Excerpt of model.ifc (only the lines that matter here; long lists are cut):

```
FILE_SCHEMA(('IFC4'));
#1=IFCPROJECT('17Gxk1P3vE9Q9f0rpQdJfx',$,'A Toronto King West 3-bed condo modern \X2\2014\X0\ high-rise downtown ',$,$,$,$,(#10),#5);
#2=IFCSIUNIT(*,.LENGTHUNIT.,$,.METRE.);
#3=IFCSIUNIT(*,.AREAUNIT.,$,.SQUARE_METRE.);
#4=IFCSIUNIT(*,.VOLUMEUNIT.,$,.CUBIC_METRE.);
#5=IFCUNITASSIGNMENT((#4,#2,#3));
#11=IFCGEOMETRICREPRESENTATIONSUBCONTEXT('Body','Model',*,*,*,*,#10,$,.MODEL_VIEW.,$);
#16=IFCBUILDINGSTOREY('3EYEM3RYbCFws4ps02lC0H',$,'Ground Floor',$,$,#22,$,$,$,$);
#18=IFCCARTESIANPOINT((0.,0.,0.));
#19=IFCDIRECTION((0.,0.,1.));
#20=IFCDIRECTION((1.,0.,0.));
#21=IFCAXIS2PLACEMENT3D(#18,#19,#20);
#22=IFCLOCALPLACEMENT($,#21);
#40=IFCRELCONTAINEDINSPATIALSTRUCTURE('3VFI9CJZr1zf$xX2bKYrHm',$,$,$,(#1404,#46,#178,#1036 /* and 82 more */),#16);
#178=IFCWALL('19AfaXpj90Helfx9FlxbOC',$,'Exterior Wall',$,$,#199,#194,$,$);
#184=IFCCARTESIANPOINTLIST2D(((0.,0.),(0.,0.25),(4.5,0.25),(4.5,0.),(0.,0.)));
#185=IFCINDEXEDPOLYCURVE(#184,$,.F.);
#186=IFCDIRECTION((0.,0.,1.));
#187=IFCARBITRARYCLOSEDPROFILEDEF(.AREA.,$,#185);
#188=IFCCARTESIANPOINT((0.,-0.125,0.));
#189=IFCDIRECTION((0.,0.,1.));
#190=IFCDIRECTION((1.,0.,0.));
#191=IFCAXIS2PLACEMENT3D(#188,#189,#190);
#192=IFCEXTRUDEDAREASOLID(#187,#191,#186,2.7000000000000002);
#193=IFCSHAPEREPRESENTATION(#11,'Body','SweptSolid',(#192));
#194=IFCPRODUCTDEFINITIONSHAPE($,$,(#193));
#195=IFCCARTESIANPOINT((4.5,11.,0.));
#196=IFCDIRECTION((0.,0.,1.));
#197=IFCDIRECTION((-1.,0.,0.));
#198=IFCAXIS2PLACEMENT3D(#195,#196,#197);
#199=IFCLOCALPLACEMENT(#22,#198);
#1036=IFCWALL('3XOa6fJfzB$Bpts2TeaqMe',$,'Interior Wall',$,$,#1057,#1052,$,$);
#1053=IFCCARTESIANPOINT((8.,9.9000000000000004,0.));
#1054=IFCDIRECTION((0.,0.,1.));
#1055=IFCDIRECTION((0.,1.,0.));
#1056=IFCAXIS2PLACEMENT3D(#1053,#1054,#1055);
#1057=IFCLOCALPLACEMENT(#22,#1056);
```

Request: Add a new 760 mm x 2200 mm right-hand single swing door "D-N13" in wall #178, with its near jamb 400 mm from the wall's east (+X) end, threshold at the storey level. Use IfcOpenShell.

```python
import numpy as np
import ifcopenshell
import ifcopenshell.api.feature
import ifcopenshell.api.geometry
import ifcopenshell.api.root
import ifcopenshell.api.spatial
import ifcopenshell.geom
import ifcopenshell.util.element
import ifcopenshell.util.placement
import ifcopenshell.util.representation
import ifcopenshell.util.shape
import ifcopenshell.util.unit

model = ifcopenshell.open("model.ifc")
unit_scale = ifcopenshell.util.unit.calculate_unit_scale(model)
settings = ifcopenshell.geom.settings()


def volume(element):
    """Net volume in cubic metres, openings subtracted."""
    shape = ifcopenshell.geom.create_shape(settings, element)
    return ifcopenshell.util.shape.get_volume(shape.geometry)


wall = model.by_guid("19AfaXpj90Helfx9FlxbOC")
storey = ifcopenshell.util.element.get_container(wall, ifc_class="IfcBuildingStorey")
context = ifcopenshell.util.representation.get_context(model, "Model", "Body", "MODEL_VIEW")
before = volume(wall)

width, height, from_end, sill = 0.76, 2.2, 0.4, 0.0  # metres

# The wall runs along its own X axis, and the end named is its -X end.
wall_shape = ifcopenshell.geom.create_shape(settings, wall)
x, y, z = ifcopenshell.util.shape.get_vertices(wall_shape.geometry).T
start = x.min() + from_end
face, thickness = float(y.min()), float(y.max() - y.min())
wall_matrix = ifcopenshell.util.placement.get_local_placement(wall.ObjectPlacement)
level = ifcopenshell.util.placement.get_local_placement(storey.ObjectPlacement)[2, 3]


def in_wall(x, y):
    """Placement at x, y metres in the wall's axes, at sill height."""
    matrix = wall_matrix.copy()
    matrix[:, 3] = wall_matrix @ np.array([x / unit_scale, y / unit_scale, 0.0, 1.0])
    matrix[2, 3] = level + sill / unit_scale
    return matrix


# Opening: a box that overshoots both wall faces by 50 mm.
opening = ifcopenshell.api.root.create_entity(model, ifc_class="IfcOpeningElement", predefined_type="OPENING")
box = ifcopenshell.api.geometry.add_wall_representation(
    model, context=context, length=width, height=height, thickness=thickness + 0.1
)
ifcopenshell.api.geometry.assign_representation(model, product=opening, representation=box)
ifcopenshell.api.geometry.edit_object_placement(model, product=opening, matrix=in_wall(start, face - 0.05), is_si=False)
ifcopenshell.api.feature.add_feature(model, feature=opening, element=wall)

door = ifcopenshell.api.root.create_entity(model, ifc_class="IfcDoor", name="D-N13", predefined_type="DOOR")
door.OverallWidth, door.OverallHeight = width / unit_scale, height / unit_scale
door.OperationType = "SINGLE_SWING_RIGHT"
body = ifcopenshell.api.geometry.add_door_representation(
    model,
    context=context,
    overall_width=door.OverallWidth,
    overall_height=door.OverallHeight,
    operation_type="SINGLE_SWING_RIGHT",
    lining_properties={"LiningDepth": thickness / unit_scale, "ThresholdDepth": thickness / unit_scale},
)
ifcopenshell.api.geometry.assign_representation(model, product=door, representation=body)
ifcopenshell.api.spatial.assign_container(model, products=[door], relating_structure=storey)
ifcopenshell.api.feature.add_filling(model, opening=opening, element=door)

# The lining spans the wall, so the door starts at the wall face.
ifcopenshell.api.geometry.edit_object_placement(model, product=door, matrix=in_wall(start, face), is_si=False)

after = volume(wall)

print(f"wall volume {before:.3f} -> {after:.3f} m3")

model.write("model_rev.ifc")
```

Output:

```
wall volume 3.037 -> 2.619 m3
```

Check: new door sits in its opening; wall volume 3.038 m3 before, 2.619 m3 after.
